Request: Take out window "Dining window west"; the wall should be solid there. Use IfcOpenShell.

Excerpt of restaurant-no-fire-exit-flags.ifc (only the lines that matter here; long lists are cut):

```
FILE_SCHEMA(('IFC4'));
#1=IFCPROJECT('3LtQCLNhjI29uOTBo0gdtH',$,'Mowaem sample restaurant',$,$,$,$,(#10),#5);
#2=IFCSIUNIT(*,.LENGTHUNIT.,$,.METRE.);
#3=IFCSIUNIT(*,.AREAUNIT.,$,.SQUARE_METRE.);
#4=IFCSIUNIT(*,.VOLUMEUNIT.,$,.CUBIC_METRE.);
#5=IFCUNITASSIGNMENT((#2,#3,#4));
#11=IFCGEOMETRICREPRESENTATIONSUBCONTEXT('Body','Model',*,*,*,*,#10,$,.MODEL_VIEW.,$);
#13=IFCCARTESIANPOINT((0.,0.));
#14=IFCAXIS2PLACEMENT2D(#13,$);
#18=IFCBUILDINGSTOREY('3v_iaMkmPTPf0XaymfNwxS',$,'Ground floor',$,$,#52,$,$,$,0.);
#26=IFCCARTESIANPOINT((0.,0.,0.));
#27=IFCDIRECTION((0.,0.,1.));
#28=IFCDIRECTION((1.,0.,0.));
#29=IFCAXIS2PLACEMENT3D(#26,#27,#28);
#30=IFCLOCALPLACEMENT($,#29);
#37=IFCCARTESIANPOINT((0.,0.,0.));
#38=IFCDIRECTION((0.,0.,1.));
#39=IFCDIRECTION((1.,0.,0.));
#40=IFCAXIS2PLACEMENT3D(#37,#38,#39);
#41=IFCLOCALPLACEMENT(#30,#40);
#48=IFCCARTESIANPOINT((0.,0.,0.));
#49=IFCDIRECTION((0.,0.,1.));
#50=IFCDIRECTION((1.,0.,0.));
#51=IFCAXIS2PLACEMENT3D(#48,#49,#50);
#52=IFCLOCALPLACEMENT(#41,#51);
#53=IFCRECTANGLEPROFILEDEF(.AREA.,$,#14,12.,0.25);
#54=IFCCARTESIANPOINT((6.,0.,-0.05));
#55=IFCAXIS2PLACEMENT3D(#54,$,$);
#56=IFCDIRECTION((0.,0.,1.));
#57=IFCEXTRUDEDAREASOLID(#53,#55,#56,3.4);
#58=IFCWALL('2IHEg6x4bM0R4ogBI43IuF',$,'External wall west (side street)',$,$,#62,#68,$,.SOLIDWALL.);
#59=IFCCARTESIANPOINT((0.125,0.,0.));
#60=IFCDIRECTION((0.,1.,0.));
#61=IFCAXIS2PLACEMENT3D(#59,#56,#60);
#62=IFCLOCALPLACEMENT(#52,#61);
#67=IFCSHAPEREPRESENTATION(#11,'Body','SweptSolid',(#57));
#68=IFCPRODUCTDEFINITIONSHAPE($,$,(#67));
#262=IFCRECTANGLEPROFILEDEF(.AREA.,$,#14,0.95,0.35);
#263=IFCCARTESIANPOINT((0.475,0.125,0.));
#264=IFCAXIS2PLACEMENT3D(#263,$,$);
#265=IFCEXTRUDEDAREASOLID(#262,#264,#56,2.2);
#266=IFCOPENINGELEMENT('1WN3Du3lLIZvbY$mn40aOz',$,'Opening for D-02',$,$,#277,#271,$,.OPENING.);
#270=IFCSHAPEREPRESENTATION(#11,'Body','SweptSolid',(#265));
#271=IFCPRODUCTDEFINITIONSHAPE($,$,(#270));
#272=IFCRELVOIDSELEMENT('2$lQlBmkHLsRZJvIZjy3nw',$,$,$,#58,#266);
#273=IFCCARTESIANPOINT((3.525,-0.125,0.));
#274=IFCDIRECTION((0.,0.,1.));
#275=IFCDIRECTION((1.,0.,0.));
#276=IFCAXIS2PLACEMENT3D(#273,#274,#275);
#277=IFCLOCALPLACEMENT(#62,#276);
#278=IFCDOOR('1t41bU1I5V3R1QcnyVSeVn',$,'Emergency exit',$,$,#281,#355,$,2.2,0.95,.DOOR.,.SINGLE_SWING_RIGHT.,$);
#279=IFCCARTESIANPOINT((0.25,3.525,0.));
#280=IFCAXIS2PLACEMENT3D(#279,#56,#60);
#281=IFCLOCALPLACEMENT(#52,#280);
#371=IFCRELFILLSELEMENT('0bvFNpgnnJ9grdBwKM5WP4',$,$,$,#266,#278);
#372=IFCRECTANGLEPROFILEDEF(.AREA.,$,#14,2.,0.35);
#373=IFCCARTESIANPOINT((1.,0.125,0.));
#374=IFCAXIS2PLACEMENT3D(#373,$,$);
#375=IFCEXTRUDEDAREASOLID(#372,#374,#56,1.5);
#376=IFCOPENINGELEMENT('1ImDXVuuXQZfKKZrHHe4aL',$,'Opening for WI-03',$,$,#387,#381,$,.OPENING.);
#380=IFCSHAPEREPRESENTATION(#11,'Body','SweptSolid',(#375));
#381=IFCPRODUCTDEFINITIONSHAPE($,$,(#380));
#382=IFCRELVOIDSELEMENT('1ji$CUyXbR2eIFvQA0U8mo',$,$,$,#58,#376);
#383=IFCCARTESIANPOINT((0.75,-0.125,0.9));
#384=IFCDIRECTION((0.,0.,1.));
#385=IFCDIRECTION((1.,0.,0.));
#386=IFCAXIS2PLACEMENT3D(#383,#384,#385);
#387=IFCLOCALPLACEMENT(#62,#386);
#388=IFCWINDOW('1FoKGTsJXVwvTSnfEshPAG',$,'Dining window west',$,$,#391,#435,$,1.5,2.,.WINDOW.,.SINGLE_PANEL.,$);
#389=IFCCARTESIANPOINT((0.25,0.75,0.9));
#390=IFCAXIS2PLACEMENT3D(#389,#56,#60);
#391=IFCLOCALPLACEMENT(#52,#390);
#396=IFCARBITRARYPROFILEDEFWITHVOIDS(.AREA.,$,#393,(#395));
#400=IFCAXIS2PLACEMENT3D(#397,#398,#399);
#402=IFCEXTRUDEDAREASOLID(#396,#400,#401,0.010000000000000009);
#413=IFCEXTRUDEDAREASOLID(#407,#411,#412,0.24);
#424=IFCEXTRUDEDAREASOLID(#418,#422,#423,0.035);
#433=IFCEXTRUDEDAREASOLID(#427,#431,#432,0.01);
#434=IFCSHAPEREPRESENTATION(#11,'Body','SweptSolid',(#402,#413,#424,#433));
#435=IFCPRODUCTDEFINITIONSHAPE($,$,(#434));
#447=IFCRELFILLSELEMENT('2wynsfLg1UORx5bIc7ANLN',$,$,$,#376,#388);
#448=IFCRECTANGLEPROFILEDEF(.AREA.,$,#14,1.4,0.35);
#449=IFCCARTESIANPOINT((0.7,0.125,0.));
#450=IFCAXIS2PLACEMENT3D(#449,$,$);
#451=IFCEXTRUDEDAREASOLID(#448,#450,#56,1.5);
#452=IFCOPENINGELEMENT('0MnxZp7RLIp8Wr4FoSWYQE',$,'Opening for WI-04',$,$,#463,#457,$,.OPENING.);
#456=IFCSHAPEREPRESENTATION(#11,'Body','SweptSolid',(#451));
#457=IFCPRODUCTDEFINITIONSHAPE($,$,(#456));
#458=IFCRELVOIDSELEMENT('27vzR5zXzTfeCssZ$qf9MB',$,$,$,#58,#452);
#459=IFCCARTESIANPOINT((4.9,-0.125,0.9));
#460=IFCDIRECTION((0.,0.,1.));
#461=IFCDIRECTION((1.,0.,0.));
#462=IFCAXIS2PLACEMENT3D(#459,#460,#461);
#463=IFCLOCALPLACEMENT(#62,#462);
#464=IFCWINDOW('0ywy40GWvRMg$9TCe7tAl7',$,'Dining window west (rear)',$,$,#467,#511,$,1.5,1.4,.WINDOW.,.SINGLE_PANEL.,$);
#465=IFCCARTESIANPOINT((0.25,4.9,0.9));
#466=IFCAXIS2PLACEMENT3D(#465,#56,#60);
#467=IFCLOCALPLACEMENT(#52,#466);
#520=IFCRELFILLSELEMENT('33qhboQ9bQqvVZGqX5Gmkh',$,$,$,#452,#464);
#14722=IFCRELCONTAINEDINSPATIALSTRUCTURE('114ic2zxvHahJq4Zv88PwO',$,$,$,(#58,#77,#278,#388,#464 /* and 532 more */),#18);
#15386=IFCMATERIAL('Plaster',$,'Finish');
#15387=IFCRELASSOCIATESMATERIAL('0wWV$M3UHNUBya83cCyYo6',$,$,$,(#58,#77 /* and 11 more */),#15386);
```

```python
import ifcopenshell
import ifcopenshell.api.feature
import ifcopenshell.api.root
import ifcopenshell.geom
import ifcopenshell.util.shape

model = ifcopenshell.open("restaurant-no-fire-exit-flags.ifc")
settings = ifcopenshell.geom.settings()


def volume(element):
    """Net volume in cubic metres, openings subtracted."""
    shape = ifcopenshell.geom.create_shape(settings, element)
    return ifcopenshell.util.shape.get_volume(shape.geometry)


window = model.by_guid("1FoKGTsJXVwvTSnfEshPAG")
opening = window.FillsVoids[0].RelatingOpeningElement
wall = opening.VoidsElements[0].RelatingBuildingElement
before = volume(wall)

ifcopenshell.api.root.remove_product(model, product=window)
ifcopenshell.api.feature.remove_feature(model, feature=opening)

after = volume(wall)

print(f"wall volume {before:.3f} -> {after:.3f} m3")

model.write("restaurant-no-fire-exit-flags_v2.ifc")
```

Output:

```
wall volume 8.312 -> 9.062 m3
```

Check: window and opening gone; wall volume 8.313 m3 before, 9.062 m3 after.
